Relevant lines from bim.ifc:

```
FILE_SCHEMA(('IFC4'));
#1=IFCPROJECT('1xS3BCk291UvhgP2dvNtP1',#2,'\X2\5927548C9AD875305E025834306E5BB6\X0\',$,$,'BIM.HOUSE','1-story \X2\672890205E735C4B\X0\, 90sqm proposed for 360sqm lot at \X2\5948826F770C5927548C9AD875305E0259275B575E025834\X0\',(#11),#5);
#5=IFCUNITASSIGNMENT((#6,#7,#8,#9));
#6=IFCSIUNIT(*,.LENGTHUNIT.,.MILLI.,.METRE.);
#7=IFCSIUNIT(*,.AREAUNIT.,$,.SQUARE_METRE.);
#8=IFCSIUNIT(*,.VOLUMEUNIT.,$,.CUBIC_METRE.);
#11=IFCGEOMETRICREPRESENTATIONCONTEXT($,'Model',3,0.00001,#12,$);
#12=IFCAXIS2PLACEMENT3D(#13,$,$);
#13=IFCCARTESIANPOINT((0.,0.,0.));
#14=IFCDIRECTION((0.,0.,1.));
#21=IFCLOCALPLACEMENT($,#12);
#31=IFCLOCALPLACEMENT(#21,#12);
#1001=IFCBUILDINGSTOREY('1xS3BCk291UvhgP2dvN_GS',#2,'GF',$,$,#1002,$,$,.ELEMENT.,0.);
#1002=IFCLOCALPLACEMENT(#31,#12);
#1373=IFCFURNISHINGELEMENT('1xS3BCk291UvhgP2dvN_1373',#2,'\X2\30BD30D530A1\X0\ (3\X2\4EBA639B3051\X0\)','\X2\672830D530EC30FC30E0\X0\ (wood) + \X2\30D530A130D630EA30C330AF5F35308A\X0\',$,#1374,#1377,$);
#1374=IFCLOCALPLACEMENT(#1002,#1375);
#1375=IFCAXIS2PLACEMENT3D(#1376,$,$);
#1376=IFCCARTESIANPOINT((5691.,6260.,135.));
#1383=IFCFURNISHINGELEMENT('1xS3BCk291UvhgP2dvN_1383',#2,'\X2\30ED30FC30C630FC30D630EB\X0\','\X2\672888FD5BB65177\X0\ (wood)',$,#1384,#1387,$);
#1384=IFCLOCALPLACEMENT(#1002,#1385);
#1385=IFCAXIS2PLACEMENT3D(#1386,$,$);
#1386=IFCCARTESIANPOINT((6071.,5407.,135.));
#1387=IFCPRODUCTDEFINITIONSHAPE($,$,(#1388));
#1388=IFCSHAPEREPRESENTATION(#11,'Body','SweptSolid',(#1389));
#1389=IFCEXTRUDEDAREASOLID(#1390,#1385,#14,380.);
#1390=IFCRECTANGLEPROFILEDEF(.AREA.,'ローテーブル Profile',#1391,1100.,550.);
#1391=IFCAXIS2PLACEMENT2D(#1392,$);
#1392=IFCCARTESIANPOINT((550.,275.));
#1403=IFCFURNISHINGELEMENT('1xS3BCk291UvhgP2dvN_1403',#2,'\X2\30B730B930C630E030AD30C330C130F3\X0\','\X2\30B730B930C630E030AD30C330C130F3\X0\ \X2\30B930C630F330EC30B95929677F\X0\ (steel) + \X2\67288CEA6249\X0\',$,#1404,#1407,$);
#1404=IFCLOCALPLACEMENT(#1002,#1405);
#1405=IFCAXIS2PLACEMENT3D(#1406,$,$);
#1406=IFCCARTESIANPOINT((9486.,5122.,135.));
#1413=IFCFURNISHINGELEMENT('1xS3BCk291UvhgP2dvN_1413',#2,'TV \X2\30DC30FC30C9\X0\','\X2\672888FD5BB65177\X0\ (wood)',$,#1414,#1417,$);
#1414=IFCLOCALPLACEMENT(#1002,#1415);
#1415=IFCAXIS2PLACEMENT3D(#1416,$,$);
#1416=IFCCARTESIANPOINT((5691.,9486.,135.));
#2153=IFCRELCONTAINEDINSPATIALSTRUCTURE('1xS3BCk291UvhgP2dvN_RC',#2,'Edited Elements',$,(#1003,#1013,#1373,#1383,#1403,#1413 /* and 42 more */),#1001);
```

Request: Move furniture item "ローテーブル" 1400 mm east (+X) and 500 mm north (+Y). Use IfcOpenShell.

```python
import ifcopenshell
import ifcopenshell.api.geometry
import ifcopenshell.util.placement

model = ifcopenshell.open("bim.ifc")

item = model.by_id(1383)
matrix = ifcopenshell.util.placement.get_local_placement(item.ObjectPlacement)
matrix[0, 3] += 1400.0
matrix[1, 3] += 500.0
ifcopenshell.api.geometry.edit_object_placement(model, product=item, matrix=matrix, is_si=False)

print(ifcopenshell.util.placement.get_local_placement(item.ObjectPlacement).round(3) + 0.0)

model.write("bim_edited.ifc")
```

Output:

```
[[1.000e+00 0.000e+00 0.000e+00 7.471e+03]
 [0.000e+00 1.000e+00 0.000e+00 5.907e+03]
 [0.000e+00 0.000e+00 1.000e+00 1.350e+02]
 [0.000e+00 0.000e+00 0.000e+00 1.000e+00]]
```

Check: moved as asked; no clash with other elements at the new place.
